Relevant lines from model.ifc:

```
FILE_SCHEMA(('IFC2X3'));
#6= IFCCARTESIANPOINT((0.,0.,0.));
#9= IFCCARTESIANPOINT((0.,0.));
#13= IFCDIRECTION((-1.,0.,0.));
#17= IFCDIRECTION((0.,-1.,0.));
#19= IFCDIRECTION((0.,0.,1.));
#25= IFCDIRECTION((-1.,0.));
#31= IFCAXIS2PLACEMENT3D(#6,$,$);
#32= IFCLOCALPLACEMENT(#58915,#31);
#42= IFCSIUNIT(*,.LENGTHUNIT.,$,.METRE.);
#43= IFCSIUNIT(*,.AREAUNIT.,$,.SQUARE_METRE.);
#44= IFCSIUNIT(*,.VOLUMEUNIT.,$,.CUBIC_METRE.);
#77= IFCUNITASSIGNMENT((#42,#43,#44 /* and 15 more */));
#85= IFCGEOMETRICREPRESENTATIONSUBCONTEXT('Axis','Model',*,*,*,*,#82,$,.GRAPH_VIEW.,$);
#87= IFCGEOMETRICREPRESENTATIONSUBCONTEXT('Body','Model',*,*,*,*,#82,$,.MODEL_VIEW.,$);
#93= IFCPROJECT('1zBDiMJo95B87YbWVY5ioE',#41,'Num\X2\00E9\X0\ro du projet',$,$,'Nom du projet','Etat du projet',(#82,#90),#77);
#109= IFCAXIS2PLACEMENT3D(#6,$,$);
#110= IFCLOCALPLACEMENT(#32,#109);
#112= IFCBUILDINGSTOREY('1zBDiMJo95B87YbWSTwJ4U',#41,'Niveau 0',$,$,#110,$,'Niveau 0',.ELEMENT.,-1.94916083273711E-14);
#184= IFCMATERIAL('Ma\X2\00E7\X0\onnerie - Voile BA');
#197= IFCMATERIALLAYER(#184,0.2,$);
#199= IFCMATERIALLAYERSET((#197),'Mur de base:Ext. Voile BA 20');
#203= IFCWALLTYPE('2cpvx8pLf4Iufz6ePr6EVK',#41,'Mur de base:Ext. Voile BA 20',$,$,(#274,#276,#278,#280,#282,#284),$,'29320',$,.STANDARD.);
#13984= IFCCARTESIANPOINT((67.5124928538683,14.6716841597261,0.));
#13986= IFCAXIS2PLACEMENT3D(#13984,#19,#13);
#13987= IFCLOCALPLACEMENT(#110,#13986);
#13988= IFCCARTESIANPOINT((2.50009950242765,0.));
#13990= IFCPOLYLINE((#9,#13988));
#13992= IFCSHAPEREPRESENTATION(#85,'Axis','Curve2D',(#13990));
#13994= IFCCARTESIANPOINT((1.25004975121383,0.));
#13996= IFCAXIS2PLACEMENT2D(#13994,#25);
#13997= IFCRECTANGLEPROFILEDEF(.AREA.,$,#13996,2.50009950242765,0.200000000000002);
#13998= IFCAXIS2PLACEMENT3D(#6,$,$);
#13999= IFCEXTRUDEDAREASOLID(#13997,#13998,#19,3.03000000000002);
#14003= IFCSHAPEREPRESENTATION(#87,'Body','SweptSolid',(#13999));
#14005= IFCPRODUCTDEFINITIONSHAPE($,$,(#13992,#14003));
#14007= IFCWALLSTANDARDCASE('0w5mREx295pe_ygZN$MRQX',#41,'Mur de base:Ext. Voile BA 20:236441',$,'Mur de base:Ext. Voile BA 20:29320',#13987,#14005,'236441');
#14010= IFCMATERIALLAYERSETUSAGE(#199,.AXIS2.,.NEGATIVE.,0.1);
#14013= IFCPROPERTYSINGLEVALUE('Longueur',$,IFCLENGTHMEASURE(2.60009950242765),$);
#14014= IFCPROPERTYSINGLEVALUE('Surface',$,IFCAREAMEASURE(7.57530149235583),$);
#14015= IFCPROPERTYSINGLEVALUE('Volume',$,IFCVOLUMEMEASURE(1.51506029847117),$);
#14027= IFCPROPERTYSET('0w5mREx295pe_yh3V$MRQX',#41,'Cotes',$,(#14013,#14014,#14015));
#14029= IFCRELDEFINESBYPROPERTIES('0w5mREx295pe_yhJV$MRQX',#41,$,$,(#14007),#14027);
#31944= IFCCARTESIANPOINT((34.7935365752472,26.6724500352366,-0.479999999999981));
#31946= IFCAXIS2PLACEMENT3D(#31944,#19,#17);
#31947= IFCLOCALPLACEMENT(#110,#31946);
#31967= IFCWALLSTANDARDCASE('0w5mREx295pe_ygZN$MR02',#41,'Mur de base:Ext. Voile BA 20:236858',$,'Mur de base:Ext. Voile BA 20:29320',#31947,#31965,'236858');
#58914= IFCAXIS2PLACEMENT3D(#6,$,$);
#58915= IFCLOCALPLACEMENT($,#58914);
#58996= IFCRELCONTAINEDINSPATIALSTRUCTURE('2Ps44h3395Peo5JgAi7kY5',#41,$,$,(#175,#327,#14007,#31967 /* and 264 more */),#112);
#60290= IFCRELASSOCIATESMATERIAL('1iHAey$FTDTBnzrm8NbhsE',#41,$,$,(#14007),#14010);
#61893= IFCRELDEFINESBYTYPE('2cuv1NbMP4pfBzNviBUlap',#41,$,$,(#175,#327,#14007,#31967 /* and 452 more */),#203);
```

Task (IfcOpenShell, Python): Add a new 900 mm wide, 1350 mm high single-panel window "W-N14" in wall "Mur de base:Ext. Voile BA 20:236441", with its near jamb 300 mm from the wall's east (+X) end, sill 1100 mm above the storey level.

```python
import numpy as np
import ifcopenshell
import ifcopenshell.api.feature
import ifcopenshell.api.geometry
import ifcopenshell.api.pset
import ifcopenshell.api.root
import ifcopenshell.api.spatial
import ifcopenshell.api.type
import ifcopenshell.geom
import ifcopenshell.util.element
import ifcopenshell.util.placement
import ifcopenshell.util.representation
import ifcopenshell.util.shape
import ifcopenshell.util.unit

model = ifcopenshell.open("model.ifc")
unit_scale = ifcopenshell.util.unit.calculate_unit_scale(model)
area_scale = ifcopenshell.util.unit.calculate_unit_scale(model, "AREAUNIT")
volume_scale = ifcopenshell.util.unit.calculate_unit_scale(model, "VOLUMEUNIT")
settings = ifcopenshell.geom.settings()


def volume(element):
    """Net volume in cubic metres, openings subtracted."""
    shape = ifcopenshell.geom.create_shape(settings, element)
    return ifcopenshell.util.shape.get_volume(shape.geometry)


wall = model.by_id(14007)
storey = ifcopenshell.util.element.get_container(wall, ifc_class="IfcBuildingStorey")
context = ifcopenshell.util.representation.get_context(model, "Model", "Body", "MODEL_VIEW")
before = volume(wall)

width, height, from_end, sill = 0.9, 1.35, 0.3, 1.1  # metres

# The wall runs along its own X axis, and the end named is its -X end.
wall_shape = ifcopenshell.geom.create_shape(settings, wall)
x, y, z = ifcopenshell.util.shape.get_vertices(wall_shape.geometry).T
start = x.min() + from_end
face, thickness = float(y.min()), float(y.max() - y.min())
wall_matrix = ifcopenshell.util.placement.get_local_placement(wall.ObjectPlacement)
level = ifcopenshell.util.placement.get_local_placement(storey.ObjectPlacement)[2, 3]


def in_wall(x, y):
    """Placement at x, y metres in the wall's axes, at sill height."""
    matrix = wall_matrix.copy()
    matrix[:, 3] = wall_matrix @ np.array([x / unit_scale, y / unit_scale, 0.0, 1.0])
    matrix[2, 3] = level + sill / unit_scale
    return matrix


# Opening: a box that overshoots both wall faces by 50 mm.
opening = ifcopenshell.api.root.create_entity(model, ifc_class="IfcOpeningElement")
box = ifcopenshell.api.geometry.add_wall_representation(
    model, context=context, length=width, height=height, thickness=thickness + 0.1
)
ifcopenshell.api.geometry.assign_representation(model, product=opening, representation=box)
ifcopenshell.api.geometry.edit_object_placement(model, product=opening, matrix=in_wall(start, face - 0.05), is_si=False)
ifcopenshell.api.feature.add_feature(model, feature=opening, element=wall)

window = ifcopenshell.api.root.create_entity(model, ifc_class="IfcWindow", name="W-N14")
window.OverallWidth, window.OverallHeight = width / unit_scale, height / unit_scale
body = ifcopenshell.api.geometry.add_window_representation(
    model,
    context=context,
    overall_width=window.OverallWidth,
    overall_height=window.OverallHeight,
    partition_type="SINGLE_PANEL",
)
ifcopenshell.api.geometry.assign_representation(model, product=window, representation=body)
ifcopenshell.api.spatial.assign_container(model, products=[window], relating_structure=storey)
fills = ifcopenshell.api.feature.add_filling(model, opening=opening, element=window)
fills.OwnerHistory = window.OwnerHistory  # required in IFC2X3

# IFC2X3 keeps the operation on the window style.
style = ifcopenshell.api.root.create_entity(model, ifc_class="IfcWindowStyle", name="W-N14")
style.OperationType, style.ConstructionType = "SINGLE_PANEL", "NOTDEFINED"
style.ParameterTakesPrecedence = style.Sizeable = False
ifcopenshell.api.type.assign_type(model, related_objects=[window], relating_type=style)

# Centre the window in the wall's thickness.
ifcopenshell.api.geometry.edit_object_placement(model, product=window, matrix=in_wall(start, face), is_si=False)
window_shape = ifcopenshell.geom.create_shape(settings, window)
depth = ifcopenshell.util.shape.get_vertices(window_shape.geometry)[:, 1]
offset = face + thickness / 2 - (depth.min() + depth.max()) / 2
ifcopenshell.api.geometry.edit_object_placement(model, product=window, matrix=in_wall(start, offset), is_si=False)

after = volume(wall)

# Update the wall's stored quantities.
pset = model.by_id(ifcopenshell.util.element.get_pset(wall, "Cotes", should_inherit=False)["id"])
ifcopenshell.api.pset.edit_pset(model, pset=pset, properties={
    "Surface": model.create_entity("IfcAreaMeasure", after / thickness / area_scale),
    "Volume": model.create_entity("IfcVolumeMeasure", after / volume_scale),
})

print(f"wall volume {before:.3f} -> {after:.3f} m3")

model.write("model-out.ifc")
```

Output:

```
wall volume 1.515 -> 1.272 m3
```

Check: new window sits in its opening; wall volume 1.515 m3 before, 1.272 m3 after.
